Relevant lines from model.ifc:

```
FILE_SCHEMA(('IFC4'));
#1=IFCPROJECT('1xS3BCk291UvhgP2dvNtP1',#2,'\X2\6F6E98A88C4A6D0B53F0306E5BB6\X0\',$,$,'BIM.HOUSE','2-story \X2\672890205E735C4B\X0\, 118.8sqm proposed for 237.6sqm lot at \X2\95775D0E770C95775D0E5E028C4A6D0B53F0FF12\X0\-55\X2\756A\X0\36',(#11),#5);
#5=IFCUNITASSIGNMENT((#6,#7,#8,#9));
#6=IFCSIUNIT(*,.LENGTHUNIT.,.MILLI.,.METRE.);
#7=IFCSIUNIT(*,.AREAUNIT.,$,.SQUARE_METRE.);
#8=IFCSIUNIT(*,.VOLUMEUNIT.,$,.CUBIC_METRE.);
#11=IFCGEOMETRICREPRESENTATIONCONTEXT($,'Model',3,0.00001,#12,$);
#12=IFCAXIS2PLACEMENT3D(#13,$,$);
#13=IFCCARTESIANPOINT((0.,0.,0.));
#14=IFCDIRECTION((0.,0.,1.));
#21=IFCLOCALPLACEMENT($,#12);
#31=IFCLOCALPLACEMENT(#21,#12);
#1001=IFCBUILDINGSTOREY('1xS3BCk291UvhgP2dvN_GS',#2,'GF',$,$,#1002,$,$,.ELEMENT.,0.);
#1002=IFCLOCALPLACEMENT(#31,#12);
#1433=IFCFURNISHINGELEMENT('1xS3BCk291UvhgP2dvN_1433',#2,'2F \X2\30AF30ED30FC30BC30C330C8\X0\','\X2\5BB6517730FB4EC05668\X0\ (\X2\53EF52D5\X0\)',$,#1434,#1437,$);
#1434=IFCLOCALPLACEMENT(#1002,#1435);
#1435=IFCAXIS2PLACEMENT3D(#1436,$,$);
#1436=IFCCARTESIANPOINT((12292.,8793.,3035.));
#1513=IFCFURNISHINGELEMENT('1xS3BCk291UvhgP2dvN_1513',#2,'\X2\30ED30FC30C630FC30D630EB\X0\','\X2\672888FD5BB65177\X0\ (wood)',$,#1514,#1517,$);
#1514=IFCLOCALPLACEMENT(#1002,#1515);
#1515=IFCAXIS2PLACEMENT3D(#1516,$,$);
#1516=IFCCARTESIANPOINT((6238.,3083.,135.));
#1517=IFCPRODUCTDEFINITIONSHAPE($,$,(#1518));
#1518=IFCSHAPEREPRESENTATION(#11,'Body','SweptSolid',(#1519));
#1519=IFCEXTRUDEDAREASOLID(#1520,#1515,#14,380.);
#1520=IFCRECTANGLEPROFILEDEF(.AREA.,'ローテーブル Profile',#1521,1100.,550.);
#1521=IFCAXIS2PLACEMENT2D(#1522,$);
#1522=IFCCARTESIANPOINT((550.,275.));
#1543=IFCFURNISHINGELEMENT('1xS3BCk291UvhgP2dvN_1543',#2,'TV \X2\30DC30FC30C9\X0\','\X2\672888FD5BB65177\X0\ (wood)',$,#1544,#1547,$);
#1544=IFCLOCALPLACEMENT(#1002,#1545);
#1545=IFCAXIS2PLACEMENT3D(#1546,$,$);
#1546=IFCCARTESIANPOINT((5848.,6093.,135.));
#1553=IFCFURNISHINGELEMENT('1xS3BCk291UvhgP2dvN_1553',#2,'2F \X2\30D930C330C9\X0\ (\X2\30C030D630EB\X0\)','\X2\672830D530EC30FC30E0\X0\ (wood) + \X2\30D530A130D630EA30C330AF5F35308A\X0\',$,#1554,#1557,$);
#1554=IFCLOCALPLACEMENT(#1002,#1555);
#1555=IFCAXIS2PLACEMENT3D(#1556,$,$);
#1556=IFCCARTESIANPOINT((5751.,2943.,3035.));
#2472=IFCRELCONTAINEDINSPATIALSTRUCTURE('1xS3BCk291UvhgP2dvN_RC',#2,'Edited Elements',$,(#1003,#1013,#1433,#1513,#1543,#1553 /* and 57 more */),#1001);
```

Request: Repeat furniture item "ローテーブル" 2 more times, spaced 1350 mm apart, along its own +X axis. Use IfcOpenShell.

```python
import ifcopenshell
import ifcopenshell.api.geometry
import ifcopenshell.api.root
import ifcopenshell.util.element
import ifcopenshell.util.placement

model = ifcopenshell.open("model.ifc")


def reuse_history(source, copy):
    """copy_class also copies each property set's owner history, people and application; keep the originals."""
    for rel in copy.IsDefinedBy:
        if rel.is_a("IfcRelDefinesByProperties") and (history := rel.RelatingPropertyDefinition.OwnerHistory):
            rel.RelatingPropertyDefinition.OwnerHistory = source.OwnerHistory
            ifcopenshell.util.element.remove_deep2(model, history)


source = model.by_id(1513)
base = ifcopenshell.util.placement.get_local_placement(source.ObjectPlacement)
step = base[:3, 0] * 1350.0

for i in range(1, 3):
    copy = ifcopenshell.api.root.copy_class(model, product=source)
    copy.Representation = ifcopenshell.util.element.copy_deep(
        model, source.Representation, exclude=["IfcGeometricRepresentationContext", "IfcRepresentationMap"]
    )
    reuse_history(source, copy)
    matrix = base.copy()
    matrix[:3, 3] += i * step
    print("added at", matrix[:3, 3].round(3) + 0.0)
    ifcopenshell.api.geometry.edit_object_placement(model, product=copy, matrix=matrix, is_si=False)

model.write("model_updated.ifc")
```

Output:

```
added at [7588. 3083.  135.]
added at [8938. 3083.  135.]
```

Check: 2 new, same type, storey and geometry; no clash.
